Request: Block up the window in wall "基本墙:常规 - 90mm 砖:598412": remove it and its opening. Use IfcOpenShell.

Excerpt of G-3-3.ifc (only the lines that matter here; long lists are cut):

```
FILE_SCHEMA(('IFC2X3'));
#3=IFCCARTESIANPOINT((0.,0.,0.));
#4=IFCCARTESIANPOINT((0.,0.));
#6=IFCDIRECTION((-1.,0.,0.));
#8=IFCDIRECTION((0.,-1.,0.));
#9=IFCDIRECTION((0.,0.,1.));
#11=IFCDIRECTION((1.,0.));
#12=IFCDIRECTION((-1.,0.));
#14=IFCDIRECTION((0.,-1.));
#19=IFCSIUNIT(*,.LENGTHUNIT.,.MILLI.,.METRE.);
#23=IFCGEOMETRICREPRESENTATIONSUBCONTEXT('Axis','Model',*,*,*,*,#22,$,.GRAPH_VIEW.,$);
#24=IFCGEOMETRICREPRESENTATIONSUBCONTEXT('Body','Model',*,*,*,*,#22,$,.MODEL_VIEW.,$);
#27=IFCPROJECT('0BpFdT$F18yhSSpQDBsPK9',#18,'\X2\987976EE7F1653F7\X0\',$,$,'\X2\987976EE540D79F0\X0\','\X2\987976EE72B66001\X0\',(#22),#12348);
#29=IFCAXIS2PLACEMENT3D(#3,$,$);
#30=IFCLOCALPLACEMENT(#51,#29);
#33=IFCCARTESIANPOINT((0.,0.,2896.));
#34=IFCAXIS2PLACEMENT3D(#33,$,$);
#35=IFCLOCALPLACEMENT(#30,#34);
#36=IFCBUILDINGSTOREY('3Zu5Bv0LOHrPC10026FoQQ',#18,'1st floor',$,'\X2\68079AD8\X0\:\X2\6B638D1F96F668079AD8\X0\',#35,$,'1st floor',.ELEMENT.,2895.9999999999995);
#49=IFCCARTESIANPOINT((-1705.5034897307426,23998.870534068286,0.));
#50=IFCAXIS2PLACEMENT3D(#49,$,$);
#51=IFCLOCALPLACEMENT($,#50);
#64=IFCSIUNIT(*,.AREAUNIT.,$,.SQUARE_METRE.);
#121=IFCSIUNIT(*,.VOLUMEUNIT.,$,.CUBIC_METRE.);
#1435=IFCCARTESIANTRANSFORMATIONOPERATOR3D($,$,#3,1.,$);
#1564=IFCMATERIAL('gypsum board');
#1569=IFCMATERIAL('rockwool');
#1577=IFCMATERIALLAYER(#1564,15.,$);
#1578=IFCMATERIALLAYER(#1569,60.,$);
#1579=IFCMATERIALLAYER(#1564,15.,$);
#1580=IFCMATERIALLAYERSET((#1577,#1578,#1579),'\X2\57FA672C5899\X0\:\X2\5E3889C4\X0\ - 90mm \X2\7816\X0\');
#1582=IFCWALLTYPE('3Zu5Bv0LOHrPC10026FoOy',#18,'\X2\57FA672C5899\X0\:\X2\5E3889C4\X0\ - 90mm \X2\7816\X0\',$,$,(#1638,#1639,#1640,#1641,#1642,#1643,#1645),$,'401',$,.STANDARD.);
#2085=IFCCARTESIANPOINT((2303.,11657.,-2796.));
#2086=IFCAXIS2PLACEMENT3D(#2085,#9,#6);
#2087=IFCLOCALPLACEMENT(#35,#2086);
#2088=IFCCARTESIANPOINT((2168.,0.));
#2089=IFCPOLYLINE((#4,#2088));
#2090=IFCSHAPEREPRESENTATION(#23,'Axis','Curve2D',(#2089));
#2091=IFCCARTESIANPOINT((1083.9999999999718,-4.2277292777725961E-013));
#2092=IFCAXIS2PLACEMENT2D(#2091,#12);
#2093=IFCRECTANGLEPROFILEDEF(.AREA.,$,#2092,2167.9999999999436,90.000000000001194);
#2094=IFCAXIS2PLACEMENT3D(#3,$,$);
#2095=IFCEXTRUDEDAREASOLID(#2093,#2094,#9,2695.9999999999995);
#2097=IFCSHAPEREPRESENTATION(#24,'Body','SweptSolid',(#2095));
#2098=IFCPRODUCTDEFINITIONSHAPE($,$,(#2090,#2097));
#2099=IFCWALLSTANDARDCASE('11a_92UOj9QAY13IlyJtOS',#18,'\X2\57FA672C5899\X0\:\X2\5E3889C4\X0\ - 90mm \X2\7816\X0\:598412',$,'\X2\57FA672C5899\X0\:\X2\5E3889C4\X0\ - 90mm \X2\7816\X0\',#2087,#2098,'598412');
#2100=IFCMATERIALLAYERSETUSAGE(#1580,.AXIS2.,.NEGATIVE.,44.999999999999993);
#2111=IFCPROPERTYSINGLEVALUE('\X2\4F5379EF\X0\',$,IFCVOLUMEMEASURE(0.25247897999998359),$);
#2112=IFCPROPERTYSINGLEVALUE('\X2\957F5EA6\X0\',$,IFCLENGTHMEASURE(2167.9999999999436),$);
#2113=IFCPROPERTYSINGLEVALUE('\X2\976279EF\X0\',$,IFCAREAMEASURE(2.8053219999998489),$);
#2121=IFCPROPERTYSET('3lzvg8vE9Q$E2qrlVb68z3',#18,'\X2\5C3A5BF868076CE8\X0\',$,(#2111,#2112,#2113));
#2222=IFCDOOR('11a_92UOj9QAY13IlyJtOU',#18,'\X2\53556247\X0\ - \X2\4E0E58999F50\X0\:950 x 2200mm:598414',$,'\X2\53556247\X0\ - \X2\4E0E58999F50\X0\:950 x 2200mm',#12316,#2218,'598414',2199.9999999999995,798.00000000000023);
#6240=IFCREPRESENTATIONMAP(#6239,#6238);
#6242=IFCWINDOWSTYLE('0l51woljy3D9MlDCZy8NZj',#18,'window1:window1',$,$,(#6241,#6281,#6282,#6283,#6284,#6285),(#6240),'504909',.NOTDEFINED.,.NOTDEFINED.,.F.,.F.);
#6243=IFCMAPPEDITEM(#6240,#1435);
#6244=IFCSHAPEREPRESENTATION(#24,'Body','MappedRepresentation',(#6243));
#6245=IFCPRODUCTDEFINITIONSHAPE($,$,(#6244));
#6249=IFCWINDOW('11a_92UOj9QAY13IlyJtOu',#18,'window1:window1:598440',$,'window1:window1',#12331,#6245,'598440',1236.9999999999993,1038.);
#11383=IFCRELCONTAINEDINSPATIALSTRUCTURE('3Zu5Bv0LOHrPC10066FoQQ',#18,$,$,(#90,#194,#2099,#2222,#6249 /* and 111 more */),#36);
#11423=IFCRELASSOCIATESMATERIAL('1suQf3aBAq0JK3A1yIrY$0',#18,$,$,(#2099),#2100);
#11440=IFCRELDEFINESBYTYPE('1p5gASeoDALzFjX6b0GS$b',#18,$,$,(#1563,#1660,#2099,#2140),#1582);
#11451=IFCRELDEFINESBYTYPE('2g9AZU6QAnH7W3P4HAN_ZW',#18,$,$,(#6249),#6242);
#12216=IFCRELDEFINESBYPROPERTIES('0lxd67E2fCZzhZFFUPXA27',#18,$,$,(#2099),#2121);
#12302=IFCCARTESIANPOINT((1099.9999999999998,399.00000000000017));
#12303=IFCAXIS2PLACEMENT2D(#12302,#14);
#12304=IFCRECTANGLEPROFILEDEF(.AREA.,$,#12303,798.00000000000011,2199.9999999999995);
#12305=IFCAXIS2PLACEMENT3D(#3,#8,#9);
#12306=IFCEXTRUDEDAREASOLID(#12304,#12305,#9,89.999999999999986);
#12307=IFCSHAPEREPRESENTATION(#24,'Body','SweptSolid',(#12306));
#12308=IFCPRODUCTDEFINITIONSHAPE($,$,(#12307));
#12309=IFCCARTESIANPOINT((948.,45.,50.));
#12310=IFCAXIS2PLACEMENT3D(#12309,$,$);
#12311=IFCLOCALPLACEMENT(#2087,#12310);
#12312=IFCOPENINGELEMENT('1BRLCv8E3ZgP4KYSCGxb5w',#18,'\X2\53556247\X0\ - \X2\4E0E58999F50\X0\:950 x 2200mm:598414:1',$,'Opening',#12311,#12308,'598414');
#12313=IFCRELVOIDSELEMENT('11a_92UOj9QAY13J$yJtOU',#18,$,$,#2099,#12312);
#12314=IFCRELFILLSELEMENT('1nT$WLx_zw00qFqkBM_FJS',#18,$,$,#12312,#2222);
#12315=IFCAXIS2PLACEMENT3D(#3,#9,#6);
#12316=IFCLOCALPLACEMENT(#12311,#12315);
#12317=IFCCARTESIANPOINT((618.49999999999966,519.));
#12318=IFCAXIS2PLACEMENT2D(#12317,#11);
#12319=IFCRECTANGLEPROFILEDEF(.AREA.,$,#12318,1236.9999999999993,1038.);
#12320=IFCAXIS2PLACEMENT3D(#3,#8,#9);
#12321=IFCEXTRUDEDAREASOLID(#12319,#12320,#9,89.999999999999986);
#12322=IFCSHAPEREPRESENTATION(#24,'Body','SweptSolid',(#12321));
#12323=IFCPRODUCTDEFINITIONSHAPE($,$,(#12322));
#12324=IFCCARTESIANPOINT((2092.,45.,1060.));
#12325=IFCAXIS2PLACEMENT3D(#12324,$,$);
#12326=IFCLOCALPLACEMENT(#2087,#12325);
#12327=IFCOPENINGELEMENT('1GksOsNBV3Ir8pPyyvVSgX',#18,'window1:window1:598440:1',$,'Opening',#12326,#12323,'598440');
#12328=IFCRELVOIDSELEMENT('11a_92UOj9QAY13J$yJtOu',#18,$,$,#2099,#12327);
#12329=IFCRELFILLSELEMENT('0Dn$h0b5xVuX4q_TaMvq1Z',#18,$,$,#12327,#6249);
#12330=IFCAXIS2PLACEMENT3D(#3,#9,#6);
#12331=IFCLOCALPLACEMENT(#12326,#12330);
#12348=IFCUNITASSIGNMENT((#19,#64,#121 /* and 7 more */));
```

```python
import ifcopenshell
import ifcopenshell.api.feature
import ifcopenshell.api.pset
import ifcopenshell.api.root
import ifcopenshell.geom
import ifcopenshell.util.element
import ifcopenshell.util.shape
import ifcopenshell.util.unit

model = ifcopenshell.open("G-3-3.ifc")
area_scale = ifcopenshell.util.unit.calculate_unit_scale(model, "AREAUNIT")
volume_scale = ifcopenshell.util.unit.calculate_unit_scale(model, "VOLUMEUNIT")
settings = ifcopenshell.geom.settings()


def volume(element):
    """Net volume in cubic metres, openings subtracted."""
    shape = ifcopenshell.geom.create_shape(settings, element)
    return ifcopenshell.util.shape.get_volume(shape.geometry)


window = model.by_id(6249)
opening = window.FillsVoids[0].RelatingOpeningElement
wall = opening.VoidsElements[0].RelatingBuildingElement
before = volume(wall)

ifcopenshell.api.root.remove_product(model, product=window)
ifcopenshell.api.feature.remove_feature(model, feature=opening)

after = volume(wall)
thickness = 0.09  # wall thickness in metres

# Update the wall's stored quantities.
pset = model.by_id(ifcopenshell.util.element.get_pset(wall, "尺寸标注", should_inherit=False)["id"])
ifcopenshell.api.pset.edit_pset(model, pset=pset, properties={
    "体积": model.create_entity("IfcVolumeMeasure", after / volume_scale),
    "面积": model.create_entity("IfcAreaMeasure", after / thickness / area_scale),
})

print(f"wall volume {before:.3f} -> {after:.3f} m3")

model.write("G-3-3_v2.ifc")
```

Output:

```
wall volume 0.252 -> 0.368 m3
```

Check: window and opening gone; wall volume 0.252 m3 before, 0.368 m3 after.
